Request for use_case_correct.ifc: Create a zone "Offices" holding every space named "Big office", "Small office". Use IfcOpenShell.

First a look at what the model holds.

```python
import ifcopenshell

model = ifcopenshell.open("use_case_correct.ifc")
print(model.schema)
seen = {}
for space in model.by_type("IfcSpace"):
    seen[space.LongName] = seen.get(space.LongName, 0) + 1
for name, count in sorted(seen.items(), key=str):
    print(count, "x", name)
print("zones:", [z.Name for z in model.by_type("IfcZone")][:20])
```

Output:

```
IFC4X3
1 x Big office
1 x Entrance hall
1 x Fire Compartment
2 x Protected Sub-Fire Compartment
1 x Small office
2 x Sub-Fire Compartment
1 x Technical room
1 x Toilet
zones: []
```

```python
import ifcopenshell
import ifcopenshell.api.group
import ifcopenshell.api.root

model = ifcopenshell.open("use_case_correct.ifc")

names = {"Big office", "Small office"}
spaces = [s for s in model.by_type("IfcSpace") if s.LongName in names]

zone = ifcopenshell.api.root.create_entity(model, ifc_class="IfcZone", name="Offices")
ifcopenshell.api.group.assign_group(model, products=spaces, group=zone)
print(len(spaces), "spaces in", zone.Name)

model.write("use_case_correct_rev.ifc")
```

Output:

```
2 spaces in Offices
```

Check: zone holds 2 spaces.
